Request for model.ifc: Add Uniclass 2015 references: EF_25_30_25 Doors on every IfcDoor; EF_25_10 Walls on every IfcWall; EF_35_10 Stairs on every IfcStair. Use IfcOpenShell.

First a look at what the model holds.

```python
import ifcopenshell

model = ifcopenshell.open("model.ifc")
print(model.schema)
print("classifications:", [c.Name for c in model.by_type("IfcClassification")])
for ifc_class in ("IfcDoor", "IfcRoof", "IfcStair", "IfcWall", "IfcWindow"):
    print(ifc_class, len(model.by_type(ifc_class)))
```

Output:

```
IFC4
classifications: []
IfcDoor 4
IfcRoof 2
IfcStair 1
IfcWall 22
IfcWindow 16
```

```python
import ifcopenshell
import ifcopenshell.api.classification

model = ifcopenshell.open("model.ifc")

system = ifcopenshell.api.classification.add_classification(model, classification="Uniclass 2015")

codes = {
    "IfcDoor": ("EF_25_30_25", "Doors"),
    "IfcWall": ("EF_25_10", "Walls"),
    "IfcStair": ("EF_35_10", "Stairs"),
}
for ifc_class, (code, name) in codes.items():
    products = model.by_type(ifc_class)
    ifcopenshell.api.classification.add_reference(
        model, products=products, classification=system, identification=code, name=name
    )
    print(code, len(products))

model.write("model-out.ifc")
```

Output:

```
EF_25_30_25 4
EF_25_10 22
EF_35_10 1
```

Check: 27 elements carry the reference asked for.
